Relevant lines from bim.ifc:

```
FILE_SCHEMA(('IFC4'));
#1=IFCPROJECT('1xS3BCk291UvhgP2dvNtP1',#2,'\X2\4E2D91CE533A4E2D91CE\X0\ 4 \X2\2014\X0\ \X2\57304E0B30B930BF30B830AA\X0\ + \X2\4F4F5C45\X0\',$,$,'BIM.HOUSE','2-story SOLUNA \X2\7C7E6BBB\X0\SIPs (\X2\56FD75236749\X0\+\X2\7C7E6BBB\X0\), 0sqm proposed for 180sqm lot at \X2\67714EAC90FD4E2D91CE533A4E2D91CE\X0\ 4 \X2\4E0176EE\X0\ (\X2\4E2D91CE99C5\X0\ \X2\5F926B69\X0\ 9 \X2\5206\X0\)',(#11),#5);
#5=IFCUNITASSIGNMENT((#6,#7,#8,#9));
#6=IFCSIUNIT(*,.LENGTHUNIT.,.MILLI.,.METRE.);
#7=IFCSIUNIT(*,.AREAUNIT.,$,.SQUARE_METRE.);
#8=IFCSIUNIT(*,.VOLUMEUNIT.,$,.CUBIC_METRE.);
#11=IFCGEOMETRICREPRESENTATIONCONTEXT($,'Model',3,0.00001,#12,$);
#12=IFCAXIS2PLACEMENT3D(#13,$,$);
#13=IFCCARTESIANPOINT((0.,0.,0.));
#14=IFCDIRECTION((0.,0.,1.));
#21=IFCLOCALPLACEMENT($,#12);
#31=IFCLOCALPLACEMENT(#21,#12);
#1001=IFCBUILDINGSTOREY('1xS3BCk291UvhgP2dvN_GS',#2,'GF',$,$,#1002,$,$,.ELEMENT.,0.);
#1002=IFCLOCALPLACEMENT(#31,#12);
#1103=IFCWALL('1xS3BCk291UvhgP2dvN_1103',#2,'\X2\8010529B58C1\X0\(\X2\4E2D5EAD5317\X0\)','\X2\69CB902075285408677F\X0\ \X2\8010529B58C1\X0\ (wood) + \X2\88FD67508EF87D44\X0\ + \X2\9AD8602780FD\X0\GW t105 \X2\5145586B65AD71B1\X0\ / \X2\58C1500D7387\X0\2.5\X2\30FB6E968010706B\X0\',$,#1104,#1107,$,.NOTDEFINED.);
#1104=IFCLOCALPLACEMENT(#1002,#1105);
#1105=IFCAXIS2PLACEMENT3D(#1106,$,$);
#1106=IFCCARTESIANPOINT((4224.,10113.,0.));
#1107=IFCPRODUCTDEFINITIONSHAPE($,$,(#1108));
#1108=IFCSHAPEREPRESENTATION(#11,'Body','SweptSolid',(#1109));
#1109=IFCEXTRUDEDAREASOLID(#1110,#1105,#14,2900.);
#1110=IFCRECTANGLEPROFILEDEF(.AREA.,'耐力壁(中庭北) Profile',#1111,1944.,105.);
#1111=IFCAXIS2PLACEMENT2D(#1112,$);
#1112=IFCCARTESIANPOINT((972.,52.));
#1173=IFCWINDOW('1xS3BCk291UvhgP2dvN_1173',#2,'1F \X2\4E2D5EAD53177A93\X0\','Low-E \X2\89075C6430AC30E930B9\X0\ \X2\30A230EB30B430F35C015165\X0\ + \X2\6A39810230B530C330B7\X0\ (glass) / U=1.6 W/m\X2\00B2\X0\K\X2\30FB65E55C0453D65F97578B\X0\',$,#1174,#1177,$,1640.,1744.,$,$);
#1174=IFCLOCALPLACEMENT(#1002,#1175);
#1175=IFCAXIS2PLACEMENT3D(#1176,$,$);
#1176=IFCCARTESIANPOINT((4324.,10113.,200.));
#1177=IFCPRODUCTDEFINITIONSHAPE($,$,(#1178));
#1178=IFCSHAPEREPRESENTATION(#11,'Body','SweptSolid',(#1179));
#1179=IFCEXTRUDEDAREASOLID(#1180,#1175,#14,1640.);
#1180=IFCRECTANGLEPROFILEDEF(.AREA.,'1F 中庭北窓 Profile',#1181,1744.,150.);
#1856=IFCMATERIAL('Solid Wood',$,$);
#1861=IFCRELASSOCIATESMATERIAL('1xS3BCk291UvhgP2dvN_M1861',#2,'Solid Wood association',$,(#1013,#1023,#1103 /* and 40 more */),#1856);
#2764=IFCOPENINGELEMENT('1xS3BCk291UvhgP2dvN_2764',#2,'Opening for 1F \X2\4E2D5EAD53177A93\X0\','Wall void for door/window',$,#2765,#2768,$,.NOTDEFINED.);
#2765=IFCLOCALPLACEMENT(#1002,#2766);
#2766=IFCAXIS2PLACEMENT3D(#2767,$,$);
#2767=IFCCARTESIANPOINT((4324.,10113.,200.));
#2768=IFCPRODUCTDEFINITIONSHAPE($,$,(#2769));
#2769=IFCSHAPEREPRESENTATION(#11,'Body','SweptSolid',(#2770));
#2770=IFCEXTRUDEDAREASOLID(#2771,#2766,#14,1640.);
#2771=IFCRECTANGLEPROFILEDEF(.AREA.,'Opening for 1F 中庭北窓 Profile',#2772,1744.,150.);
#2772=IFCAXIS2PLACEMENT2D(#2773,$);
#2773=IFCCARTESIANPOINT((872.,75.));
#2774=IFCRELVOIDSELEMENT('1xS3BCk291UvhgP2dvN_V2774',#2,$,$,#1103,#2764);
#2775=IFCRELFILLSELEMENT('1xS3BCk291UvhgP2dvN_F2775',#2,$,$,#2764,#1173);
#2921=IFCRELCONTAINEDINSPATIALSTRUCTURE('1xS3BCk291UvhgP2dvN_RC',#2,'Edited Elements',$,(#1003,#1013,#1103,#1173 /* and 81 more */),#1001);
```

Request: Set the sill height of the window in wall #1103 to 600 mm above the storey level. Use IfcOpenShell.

```python
import numpy as np
import ifcopenshell
import ifcopenshell.api.geometry
import ifcopenshell.geom
import ifcopenshell.util.element
import ifcopenshell.util.placement
import ifcopenshell.util.shape
import ifcopenshell.util.unit

model = ifcopenshell.open("bim.ifc")
unit_scale = ifcopenshell.util.unit.calculate_unit_scale(model)

window = model.by_id(1173)
opening = window.FillsVoids[0].RelatingOpeningElement
storey = ifcopenshell.util.element.get_container(window, ifc_class="IfcBuildingStorey")
level = ifcopenshell.util.placement.get_local_placement(storey.ObjectPlacement)[2, 3]

# The opening's origin need not be at the sill, so measure its lowest point.
shape = ifcopenshell.geom.create_shape(ifcopenshell.geom.settings(), opening)
bottom = ifcopenshell.util.shape.get_shape_bottom_elevation(shape, shape.geometry) / unit_scale
dz = level + 0.6 / unit_scale - bottom

shift = np.array([0.0, 0.0, dz])
# The window is not placed relative to its opening, so move both.
for product in (opening, window):
    matrix = ifcopenshell.util.placement.get_local_placement(product.ObjectPlacement)
    matrix[:3, 3] += shift
    ifcopenshell.api.geometry.edit_object_placement(model, product=product, matrix=matrix, is_si=False)

print(f"moved by {dz * unit_scale:+.3f} m")

model.write("bim-out.ifc")
```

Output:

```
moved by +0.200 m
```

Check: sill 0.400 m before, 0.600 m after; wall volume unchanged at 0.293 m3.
